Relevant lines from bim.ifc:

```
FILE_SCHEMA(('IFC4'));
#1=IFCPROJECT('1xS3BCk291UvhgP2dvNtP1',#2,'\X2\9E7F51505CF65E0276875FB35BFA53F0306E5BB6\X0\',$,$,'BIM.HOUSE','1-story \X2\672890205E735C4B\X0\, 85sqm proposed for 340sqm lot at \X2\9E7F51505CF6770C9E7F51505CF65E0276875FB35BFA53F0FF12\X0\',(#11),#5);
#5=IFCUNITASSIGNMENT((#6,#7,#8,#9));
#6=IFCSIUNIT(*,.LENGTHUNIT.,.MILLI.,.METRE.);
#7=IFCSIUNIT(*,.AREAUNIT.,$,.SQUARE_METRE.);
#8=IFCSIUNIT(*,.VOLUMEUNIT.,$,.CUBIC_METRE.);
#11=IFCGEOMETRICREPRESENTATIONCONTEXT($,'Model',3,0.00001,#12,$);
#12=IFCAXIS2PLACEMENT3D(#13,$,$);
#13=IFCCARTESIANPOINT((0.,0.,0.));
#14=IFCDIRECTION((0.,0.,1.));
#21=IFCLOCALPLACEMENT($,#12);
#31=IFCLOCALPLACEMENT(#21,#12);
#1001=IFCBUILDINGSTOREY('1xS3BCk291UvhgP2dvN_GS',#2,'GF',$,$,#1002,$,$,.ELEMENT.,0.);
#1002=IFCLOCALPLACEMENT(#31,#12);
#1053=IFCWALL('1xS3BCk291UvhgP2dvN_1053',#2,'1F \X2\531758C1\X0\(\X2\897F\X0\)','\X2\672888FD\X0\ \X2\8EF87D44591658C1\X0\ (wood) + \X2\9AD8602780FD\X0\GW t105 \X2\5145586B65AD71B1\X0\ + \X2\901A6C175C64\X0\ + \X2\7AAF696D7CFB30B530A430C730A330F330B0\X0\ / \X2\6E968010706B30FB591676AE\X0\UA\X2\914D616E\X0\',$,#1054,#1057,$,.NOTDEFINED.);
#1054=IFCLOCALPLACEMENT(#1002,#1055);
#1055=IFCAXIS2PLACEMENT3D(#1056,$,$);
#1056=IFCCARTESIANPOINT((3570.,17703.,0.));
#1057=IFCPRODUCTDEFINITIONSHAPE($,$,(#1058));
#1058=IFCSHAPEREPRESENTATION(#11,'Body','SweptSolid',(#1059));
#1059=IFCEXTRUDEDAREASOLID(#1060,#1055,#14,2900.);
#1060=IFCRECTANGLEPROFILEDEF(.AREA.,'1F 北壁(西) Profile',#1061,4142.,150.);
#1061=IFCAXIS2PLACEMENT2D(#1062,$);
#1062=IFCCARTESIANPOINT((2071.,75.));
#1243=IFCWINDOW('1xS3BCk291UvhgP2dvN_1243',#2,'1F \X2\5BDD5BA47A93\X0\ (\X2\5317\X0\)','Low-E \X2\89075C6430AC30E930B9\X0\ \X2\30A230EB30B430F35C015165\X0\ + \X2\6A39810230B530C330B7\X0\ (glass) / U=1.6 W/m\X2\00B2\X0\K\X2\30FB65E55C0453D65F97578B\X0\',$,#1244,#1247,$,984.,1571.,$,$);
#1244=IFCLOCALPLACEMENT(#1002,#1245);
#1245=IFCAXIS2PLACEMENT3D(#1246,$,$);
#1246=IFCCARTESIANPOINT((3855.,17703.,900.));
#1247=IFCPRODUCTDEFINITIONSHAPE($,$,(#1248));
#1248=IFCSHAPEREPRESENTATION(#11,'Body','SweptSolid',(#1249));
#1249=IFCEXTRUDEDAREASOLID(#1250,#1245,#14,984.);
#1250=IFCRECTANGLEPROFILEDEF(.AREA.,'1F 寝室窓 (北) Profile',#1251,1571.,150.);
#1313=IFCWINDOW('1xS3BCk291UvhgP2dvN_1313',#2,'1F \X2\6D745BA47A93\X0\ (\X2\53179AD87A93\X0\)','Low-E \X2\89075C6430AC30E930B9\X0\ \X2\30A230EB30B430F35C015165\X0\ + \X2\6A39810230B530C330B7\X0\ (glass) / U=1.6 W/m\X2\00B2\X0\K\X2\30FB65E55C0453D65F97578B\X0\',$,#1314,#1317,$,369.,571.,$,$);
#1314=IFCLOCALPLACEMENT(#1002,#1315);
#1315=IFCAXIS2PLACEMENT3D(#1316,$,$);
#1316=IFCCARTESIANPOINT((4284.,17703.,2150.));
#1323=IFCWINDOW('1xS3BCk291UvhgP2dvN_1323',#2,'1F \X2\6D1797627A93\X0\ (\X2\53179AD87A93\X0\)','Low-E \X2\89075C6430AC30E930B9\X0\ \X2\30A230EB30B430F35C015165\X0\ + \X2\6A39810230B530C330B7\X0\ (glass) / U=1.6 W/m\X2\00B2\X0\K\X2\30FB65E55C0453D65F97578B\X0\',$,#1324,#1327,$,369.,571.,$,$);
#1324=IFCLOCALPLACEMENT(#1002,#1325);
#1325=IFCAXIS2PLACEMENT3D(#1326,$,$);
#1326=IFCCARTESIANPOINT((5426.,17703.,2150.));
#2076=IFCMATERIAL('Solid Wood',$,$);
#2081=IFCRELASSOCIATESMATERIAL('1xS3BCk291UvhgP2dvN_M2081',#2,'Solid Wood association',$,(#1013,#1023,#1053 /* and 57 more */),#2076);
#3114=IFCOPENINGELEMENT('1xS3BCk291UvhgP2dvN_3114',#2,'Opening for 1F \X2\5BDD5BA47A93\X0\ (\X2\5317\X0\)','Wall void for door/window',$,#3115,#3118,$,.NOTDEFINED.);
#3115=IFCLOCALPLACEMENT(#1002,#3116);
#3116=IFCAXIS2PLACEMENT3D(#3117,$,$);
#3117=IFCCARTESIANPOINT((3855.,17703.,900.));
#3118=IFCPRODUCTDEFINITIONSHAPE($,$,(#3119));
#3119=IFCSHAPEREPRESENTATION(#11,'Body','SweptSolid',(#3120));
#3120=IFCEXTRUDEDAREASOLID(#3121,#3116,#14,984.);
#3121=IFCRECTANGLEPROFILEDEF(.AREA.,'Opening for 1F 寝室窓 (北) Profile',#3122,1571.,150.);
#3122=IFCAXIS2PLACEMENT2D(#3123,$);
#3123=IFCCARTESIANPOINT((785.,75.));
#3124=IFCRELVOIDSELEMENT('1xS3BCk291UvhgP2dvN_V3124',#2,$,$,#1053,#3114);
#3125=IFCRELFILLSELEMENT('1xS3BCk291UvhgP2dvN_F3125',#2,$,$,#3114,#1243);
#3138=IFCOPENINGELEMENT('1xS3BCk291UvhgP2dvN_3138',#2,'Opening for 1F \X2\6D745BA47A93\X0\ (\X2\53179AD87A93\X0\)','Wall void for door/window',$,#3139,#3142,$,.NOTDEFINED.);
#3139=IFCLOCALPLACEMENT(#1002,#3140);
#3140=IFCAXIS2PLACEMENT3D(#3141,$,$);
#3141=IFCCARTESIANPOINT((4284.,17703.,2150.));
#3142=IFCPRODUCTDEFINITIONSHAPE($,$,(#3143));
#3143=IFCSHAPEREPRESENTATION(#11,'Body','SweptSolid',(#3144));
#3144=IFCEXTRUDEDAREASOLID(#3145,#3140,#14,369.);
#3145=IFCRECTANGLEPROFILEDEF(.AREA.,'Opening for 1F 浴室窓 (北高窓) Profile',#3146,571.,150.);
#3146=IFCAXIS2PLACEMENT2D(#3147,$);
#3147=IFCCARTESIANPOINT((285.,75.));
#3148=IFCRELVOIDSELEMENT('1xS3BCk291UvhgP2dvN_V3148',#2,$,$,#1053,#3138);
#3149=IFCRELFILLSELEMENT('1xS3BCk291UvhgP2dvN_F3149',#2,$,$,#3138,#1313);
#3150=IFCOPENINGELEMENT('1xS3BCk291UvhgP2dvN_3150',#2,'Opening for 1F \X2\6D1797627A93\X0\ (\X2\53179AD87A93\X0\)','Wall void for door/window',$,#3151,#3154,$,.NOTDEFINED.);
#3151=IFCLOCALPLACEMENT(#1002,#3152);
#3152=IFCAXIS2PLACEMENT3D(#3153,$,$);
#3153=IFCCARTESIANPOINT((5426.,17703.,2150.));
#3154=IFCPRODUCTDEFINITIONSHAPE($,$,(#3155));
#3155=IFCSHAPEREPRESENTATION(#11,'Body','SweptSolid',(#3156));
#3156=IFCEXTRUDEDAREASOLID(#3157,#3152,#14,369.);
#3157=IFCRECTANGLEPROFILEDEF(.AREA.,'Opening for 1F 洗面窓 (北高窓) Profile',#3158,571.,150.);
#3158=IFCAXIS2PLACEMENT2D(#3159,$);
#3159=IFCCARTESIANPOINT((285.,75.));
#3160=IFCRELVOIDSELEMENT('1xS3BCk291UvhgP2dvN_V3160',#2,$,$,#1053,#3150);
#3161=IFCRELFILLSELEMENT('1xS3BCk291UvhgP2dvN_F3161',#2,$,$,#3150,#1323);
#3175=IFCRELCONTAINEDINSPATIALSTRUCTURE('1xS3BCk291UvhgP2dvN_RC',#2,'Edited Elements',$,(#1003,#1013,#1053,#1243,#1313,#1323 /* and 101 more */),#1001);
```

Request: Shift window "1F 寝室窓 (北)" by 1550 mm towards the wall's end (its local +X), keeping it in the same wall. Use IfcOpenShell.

```python
import ifcopenshell
import ifcopenshell.api.geometry
import ifcopenshell.util.placement
import ifcopenshell.util.unit

model = ifcopenshell.open("bim.ifc")
unit_scale = ifcopenshell.util.unit.calculate_unit_scale(model)

window = model.by_id(1243)
opening = window.FillsVoids[0].RelatingOpeningElement
wall = opening.VoidsElements[0].RelatingBuildingElement

wall_matrix = ifcopenshell.util.placement.get_local_placement(wall.ObjectPlacement)
shift = wall_matrix[:3, 0] * 1.55 / unit_scale
before = ifcopenshell.util.placement.get_local_placement(window.ObjectPlacement)[:3, 3].copy()

# The window is not placed relative to its opening, so move both.
for product in (opening, window):
    matrix = ifcopenshell.util.placement.get_local_placement(product.ObjectPlacement)
    matrix[:3, 3] += shift
    ifcopenshell.api.geometry.edit_object_placement(model, product=product, matrix=matrix, is_si=False)

after = ifcopenshell.util.placement.get_local_placement(window.ObjectPlacement)[:3, 3]
print("window moved by", (after - before).round(3) + 0.0)

model.write("bim_v2.ifc")
```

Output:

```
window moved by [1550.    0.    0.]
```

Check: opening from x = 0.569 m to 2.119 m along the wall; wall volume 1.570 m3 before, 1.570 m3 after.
